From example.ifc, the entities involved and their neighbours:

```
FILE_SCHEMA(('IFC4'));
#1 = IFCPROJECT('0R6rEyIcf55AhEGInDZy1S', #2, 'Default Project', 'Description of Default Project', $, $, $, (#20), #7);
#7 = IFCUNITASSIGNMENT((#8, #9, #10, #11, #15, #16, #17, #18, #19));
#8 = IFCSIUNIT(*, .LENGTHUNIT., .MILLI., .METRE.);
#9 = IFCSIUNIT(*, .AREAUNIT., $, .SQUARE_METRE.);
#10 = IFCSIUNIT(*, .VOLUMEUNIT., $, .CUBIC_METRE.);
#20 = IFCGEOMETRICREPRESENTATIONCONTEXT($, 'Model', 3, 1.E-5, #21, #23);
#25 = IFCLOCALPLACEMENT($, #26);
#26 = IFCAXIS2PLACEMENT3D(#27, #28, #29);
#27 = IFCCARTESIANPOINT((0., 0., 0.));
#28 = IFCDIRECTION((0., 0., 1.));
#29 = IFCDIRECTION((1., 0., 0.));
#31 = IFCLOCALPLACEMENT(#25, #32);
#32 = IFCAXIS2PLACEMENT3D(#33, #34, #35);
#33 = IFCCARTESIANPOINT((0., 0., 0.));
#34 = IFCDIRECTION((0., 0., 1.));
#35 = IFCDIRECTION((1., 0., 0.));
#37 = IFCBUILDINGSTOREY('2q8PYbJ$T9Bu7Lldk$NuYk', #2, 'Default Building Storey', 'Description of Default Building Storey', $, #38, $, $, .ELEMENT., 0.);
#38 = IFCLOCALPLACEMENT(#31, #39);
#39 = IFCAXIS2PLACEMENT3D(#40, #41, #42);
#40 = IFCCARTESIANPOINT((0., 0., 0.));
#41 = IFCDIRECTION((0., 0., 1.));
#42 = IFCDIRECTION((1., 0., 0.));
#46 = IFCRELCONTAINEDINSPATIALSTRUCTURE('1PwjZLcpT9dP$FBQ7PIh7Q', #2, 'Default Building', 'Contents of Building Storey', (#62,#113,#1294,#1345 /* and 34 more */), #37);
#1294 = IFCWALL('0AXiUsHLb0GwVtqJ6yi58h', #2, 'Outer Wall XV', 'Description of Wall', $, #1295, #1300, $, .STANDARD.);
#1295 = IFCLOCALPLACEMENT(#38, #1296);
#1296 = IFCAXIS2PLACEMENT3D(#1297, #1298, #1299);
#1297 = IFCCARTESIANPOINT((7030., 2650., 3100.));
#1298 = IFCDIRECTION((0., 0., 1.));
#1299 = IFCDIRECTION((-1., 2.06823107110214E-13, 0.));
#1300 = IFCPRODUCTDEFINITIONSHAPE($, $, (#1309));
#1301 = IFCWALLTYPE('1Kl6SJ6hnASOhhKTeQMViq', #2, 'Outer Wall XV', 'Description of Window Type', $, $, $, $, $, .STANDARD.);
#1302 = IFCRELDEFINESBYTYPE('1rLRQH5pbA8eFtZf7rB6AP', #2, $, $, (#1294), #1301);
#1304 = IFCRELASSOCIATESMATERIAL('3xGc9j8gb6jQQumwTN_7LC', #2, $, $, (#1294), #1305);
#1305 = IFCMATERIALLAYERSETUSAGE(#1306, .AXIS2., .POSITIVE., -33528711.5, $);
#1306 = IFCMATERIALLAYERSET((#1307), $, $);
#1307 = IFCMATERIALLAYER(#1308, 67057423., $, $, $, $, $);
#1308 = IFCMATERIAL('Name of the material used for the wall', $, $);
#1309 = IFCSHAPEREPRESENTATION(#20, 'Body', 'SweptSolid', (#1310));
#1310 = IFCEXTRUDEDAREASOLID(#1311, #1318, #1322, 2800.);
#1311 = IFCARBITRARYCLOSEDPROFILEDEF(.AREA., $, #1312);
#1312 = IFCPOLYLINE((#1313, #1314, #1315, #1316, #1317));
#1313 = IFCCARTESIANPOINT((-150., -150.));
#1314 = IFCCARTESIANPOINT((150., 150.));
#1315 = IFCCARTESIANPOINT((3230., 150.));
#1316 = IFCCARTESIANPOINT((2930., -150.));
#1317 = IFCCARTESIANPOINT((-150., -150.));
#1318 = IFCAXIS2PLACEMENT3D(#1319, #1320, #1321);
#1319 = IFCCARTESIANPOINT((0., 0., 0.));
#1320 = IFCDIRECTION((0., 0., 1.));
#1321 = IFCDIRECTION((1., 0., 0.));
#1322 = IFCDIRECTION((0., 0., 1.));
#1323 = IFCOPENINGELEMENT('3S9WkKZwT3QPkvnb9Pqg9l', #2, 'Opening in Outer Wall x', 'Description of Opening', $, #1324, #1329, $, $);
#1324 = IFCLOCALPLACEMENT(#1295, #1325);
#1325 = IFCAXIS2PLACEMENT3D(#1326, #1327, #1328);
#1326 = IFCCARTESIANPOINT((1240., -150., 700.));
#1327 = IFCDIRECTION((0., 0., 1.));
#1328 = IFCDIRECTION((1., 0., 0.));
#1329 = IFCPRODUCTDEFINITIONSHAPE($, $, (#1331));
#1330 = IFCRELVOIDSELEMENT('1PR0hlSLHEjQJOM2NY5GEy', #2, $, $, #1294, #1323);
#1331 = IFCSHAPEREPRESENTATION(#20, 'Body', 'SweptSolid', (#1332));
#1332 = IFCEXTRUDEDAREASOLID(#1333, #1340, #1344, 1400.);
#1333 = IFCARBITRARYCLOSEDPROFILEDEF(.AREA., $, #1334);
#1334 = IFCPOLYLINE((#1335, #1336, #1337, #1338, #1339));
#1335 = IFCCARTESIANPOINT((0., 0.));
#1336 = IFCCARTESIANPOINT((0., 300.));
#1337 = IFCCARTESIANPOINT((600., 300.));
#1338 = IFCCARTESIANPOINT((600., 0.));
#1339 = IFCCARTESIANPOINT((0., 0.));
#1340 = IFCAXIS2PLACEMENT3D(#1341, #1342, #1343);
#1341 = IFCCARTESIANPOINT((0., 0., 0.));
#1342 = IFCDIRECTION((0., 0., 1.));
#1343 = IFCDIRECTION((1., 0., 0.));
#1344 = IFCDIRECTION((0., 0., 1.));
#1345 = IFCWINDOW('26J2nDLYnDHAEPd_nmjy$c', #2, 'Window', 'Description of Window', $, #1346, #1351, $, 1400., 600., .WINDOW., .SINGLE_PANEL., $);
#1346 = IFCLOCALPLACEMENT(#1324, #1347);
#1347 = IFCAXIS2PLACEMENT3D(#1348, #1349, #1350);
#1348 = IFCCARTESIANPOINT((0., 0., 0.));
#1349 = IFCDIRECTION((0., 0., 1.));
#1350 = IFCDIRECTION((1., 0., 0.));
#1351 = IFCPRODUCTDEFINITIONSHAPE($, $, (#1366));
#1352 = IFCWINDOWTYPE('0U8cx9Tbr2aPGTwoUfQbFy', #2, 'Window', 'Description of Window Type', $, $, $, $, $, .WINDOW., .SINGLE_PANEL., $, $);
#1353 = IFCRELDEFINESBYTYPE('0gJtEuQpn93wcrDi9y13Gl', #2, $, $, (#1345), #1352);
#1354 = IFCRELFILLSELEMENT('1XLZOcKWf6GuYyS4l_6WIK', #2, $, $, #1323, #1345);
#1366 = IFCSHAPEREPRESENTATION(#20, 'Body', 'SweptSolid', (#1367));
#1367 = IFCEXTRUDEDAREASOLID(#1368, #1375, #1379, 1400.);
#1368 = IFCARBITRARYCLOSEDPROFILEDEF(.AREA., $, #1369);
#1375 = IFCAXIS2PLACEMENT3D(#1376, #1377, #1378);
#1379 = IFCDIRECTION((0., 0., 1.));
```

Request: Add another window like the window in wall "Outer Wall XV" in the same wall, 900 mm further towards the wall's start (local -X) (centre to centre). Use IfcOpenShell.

```python
import ifcopenshell
import ifcopenshell.api.feature
import ifcopenshell.api.geometry
import ifcopenshell.api.root
import ifcopenshell.geom
import ifcopenshell.util.element
import ifcopenshell.util.placement
import ifcopenshell.util.shape

model = ifcopenshell.open("example.ifc")
settings = ifcopenshell.geom.settings()


def volume(element):
    """Net volume in cubic metres, openings subtracted."""
    shape = ifcopenshell.geom.create_shape(settings, element)
    return ifcopenshell.util.shape.get_volume(shape.geometry)


def reuse_history(source, copy):
    """copy_class also copies each property set's owner history, people and application; keep the originals."""
    for rel in copy.IsDefinedBy:
        if rel.is_a("IfcRelDefinesByProperties") and (history := rel.RelatingPropertyDefinition.OwnerHistory):
            rel.RelatingPropertyDefinition.OwnerHistory = source.OwnerHistory
            ifcopenshell.util.element.remove_deep2(model, history)


window = model.by_guid("26J2nDLYnDHAEPd_nmjy$c")
opening = window.FillsVoids[0].RelatingOpeningElement
wall = opening.VoidsElements[0].RelatingBuildingElement
before = volume(wall)
shift = ifcopenshell.util.placement.get_local_placement(wall.ObjectPlacement)[:3, 0] * -900.0

# copy_class copies the void relationship, type, container and properties, but no geometry.
new_opening = ifcopenshell.api.root.copy_class(model, product=opening)
new_opening.Representation = ifcopenshell.util.element.copy_deep(
    model, opening.Representation, exclude=["IfcGeometricRepresentationContext", "IfcRepresentationMap"]
)
new_window = ifcopenshell.api.root.copy_class(model, product=window)
new_window.Representation = ifcopenshell.util.element.copy_deep(
    model, window.Representation, exclude=["IfcGeometricRepresentationContext", "IfcRepresentationMap"]
)
reuse_history(window, new_window)
ifcopenshell.api.feature.add_filling(model, opening=new_opening, element=new_window)

for old, new in ((opening, new_opening), (window, new_window)):
    matrix = ifcopenshell.util.placement.get_local_placement(old.ObjectPlacement)
    matrix[:3, 3] += shift
    ifcopenshell.api.geometry.edit_object_placement(model, product=new, matrix=matrix, is_si=False)

after = volume(wall)

print(f"wall volume {before:.3f} -> {after:.3f} m3")

model.write("example_edited.ifc")
```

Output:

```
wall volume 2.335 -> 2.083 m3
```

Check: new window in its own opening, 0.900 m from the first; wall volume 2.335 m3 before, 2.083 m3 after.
